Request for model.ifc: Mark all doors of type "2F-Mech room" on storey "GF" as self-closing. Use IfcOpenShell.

First a look at what the model holds.

```python
import ifcopenshell
import ifcopenshell.util.element

model = ifcopenshell.open("model.ifc")
print(model.schema)
storey = next(s for s in model.by_type("IfcBuildingStorey") if s.Name == "GF")
doors = [e for e in ifcopenshell.util.element.get_decomposition(storey) if e.is_a("IfcDoor")]
seen = {}
for e in doors:
    element_type = ifcopenshell.util.element.get_type(e)
    key = (element_type.Name if element_type != e and element_type else None, ifcopenshell.util.element.get_pset(e, "Pset_DoorCommon", "SelfClosing"))
    seen[key] = seen.get(key, 0) + 1
for (name, value), count in sorted(seen.items(), key=str):
    print(count, "x", name, "|", value)
```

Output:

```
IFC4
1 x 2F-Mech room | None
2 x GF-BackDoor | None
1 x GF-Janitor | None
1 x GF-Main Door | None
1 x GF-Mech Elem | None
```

```python
import ifcopenshell
import ifcopenshell.api.pset
import ifcopenshell.util.element

model = ifcopenshell.open("model.ifc")

storey = next(s for s in model.by_type("IfcBuildingStorey") if s.Name == "GF")
doors = [e for e in ifcopenshell.util.element.get_decomposition(storey) if e.is_a("IfcDoor")]

count = 0
for e in doors:
    element_type = ifcopenshell.util.element.get_type(e)
    if element_type in (None, e) or element_type.Name != "2F-Mech room":
        continue
    # add_pset returns the element's existing set when there is one.
    pset = ifcopenshell.api.pset.add_pset(model, product=e, name="Pset_DoorCommon")
    ifcopenshell.api.pset.edit_pset(model, pset=pset, properties={"SelfClosing": True})
    count += 1

print(count, "doors updated")

model.write("model_v2.ifc")
```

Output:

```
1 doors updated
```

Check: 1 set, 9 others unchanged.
